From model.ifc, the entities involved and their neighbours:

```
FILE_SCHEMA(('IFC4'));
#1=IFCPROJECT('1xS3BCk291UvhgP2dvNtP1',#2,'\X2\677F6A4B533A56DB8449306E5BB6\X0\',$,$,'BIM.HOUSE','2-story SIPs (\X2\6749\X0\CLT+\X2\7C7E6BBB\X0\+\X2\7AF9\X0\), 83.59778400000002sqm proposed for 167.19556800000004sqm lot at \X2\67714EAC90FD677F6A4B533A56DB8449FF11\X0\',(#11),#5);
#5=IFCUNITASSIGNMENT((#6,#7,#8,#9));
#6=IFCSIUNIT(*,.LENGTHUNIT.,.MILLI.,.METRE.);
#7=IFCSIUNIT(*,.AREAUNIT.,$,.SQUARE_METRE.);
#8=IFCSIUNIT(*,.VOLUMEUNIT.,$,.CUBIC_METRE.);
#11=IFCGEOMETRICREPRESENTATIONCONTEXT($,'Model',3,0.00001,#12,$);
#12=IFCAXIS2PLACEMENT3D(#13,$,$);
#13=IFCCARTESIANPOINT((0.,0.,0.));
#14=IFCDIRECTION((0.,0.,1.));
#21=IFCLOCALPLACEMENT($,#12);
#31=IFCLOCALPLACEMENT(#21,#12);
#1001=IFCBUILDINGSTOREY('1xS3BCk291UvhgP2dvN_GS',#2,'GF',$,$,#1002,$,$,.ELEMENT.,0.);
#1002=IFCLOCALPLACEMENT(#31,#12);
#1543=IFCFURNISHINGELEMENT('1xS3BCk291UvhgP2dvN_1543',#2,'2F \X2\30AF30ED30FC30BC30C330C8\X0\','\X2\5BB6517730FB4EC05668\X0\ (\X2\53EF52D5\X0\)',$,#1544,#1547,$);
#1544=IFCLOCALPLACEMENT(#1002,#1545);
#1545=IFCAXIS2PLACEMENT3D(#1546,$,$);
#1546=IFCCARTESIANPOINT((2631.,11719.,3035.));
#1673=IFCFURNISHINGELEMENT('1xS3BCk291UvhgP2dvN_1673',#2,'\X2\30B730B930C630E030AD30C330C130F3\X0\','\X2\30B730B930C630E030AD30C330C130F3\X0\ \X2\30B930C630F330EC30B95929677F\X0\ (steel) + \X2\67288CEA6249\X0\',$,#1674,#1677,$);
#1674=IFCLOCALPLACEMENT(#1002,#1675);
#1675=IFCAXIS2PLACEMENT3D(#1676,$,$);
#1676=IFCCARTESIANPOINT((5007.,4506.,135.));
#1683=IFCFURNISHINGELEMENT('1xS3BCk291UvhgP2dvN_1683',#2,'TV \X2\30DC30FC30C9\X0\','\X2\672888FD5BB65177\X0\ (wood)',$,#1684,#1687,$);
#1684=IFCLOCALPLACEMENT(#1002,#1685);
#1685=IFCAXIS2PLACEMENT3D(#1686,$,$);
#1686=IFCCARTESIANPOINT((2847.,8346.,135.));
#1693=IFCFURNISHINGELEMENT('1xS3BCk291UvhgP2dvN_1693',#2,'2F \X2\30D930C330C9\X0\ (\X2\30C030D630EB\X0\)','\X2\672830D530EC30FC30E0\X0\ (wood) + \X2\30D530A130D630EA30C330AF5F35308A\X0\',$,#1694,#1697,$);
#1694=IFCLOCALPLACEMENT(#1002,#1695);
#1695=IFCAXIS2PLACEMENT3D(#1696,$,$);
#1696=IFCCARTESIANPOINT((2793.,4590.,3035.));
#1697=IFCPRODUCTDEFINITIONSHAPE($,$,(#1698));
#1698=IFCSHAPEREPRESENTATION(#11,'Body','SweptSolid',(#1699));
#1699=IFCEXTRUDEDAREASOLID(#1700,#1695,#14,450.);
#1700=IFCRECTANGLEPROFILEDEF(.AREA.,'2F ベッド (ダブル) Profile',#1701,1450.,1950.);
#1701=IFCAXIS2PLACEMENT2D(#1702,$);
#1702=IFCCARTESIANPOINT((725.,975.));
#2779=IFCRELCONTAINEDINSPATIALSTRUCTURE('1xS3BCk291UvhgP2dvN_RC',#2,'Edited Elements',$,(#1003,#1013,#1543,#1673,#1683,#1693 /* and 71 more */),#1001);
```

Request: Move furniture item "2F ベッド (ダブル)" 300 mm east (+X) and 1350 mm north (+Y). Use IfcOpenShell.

```python
import ifcopenshell
import ifcopenshell.api.geometry
import ifcopenshell.util.placement

model = ifcopenshell.open("model.ifc")

item = model.by_id(1693)
matrix = ifcopenshell.util.placement.get_local_placement(item.ObjectPlacement)
matrix[0, 3] += 300.0
matrix[1, 3] += 1350.0
ifcopenshell.api.geometry.edit_object_placement(model, product=item, matrix=matrix, is_si=False)

print(ifcopenshell.util.placement.get_local_placement(item.ObjectPlacement).round(3) + 0.0)

model.write("model_v2.ifc")
```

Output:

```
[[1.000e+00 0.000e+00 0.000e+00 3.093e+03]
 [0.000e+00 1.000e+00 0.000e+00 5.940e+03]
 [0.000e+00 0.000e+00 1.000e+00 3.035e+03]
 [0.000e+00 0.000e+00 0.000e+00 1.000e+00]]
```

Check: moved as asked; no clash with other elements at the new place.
